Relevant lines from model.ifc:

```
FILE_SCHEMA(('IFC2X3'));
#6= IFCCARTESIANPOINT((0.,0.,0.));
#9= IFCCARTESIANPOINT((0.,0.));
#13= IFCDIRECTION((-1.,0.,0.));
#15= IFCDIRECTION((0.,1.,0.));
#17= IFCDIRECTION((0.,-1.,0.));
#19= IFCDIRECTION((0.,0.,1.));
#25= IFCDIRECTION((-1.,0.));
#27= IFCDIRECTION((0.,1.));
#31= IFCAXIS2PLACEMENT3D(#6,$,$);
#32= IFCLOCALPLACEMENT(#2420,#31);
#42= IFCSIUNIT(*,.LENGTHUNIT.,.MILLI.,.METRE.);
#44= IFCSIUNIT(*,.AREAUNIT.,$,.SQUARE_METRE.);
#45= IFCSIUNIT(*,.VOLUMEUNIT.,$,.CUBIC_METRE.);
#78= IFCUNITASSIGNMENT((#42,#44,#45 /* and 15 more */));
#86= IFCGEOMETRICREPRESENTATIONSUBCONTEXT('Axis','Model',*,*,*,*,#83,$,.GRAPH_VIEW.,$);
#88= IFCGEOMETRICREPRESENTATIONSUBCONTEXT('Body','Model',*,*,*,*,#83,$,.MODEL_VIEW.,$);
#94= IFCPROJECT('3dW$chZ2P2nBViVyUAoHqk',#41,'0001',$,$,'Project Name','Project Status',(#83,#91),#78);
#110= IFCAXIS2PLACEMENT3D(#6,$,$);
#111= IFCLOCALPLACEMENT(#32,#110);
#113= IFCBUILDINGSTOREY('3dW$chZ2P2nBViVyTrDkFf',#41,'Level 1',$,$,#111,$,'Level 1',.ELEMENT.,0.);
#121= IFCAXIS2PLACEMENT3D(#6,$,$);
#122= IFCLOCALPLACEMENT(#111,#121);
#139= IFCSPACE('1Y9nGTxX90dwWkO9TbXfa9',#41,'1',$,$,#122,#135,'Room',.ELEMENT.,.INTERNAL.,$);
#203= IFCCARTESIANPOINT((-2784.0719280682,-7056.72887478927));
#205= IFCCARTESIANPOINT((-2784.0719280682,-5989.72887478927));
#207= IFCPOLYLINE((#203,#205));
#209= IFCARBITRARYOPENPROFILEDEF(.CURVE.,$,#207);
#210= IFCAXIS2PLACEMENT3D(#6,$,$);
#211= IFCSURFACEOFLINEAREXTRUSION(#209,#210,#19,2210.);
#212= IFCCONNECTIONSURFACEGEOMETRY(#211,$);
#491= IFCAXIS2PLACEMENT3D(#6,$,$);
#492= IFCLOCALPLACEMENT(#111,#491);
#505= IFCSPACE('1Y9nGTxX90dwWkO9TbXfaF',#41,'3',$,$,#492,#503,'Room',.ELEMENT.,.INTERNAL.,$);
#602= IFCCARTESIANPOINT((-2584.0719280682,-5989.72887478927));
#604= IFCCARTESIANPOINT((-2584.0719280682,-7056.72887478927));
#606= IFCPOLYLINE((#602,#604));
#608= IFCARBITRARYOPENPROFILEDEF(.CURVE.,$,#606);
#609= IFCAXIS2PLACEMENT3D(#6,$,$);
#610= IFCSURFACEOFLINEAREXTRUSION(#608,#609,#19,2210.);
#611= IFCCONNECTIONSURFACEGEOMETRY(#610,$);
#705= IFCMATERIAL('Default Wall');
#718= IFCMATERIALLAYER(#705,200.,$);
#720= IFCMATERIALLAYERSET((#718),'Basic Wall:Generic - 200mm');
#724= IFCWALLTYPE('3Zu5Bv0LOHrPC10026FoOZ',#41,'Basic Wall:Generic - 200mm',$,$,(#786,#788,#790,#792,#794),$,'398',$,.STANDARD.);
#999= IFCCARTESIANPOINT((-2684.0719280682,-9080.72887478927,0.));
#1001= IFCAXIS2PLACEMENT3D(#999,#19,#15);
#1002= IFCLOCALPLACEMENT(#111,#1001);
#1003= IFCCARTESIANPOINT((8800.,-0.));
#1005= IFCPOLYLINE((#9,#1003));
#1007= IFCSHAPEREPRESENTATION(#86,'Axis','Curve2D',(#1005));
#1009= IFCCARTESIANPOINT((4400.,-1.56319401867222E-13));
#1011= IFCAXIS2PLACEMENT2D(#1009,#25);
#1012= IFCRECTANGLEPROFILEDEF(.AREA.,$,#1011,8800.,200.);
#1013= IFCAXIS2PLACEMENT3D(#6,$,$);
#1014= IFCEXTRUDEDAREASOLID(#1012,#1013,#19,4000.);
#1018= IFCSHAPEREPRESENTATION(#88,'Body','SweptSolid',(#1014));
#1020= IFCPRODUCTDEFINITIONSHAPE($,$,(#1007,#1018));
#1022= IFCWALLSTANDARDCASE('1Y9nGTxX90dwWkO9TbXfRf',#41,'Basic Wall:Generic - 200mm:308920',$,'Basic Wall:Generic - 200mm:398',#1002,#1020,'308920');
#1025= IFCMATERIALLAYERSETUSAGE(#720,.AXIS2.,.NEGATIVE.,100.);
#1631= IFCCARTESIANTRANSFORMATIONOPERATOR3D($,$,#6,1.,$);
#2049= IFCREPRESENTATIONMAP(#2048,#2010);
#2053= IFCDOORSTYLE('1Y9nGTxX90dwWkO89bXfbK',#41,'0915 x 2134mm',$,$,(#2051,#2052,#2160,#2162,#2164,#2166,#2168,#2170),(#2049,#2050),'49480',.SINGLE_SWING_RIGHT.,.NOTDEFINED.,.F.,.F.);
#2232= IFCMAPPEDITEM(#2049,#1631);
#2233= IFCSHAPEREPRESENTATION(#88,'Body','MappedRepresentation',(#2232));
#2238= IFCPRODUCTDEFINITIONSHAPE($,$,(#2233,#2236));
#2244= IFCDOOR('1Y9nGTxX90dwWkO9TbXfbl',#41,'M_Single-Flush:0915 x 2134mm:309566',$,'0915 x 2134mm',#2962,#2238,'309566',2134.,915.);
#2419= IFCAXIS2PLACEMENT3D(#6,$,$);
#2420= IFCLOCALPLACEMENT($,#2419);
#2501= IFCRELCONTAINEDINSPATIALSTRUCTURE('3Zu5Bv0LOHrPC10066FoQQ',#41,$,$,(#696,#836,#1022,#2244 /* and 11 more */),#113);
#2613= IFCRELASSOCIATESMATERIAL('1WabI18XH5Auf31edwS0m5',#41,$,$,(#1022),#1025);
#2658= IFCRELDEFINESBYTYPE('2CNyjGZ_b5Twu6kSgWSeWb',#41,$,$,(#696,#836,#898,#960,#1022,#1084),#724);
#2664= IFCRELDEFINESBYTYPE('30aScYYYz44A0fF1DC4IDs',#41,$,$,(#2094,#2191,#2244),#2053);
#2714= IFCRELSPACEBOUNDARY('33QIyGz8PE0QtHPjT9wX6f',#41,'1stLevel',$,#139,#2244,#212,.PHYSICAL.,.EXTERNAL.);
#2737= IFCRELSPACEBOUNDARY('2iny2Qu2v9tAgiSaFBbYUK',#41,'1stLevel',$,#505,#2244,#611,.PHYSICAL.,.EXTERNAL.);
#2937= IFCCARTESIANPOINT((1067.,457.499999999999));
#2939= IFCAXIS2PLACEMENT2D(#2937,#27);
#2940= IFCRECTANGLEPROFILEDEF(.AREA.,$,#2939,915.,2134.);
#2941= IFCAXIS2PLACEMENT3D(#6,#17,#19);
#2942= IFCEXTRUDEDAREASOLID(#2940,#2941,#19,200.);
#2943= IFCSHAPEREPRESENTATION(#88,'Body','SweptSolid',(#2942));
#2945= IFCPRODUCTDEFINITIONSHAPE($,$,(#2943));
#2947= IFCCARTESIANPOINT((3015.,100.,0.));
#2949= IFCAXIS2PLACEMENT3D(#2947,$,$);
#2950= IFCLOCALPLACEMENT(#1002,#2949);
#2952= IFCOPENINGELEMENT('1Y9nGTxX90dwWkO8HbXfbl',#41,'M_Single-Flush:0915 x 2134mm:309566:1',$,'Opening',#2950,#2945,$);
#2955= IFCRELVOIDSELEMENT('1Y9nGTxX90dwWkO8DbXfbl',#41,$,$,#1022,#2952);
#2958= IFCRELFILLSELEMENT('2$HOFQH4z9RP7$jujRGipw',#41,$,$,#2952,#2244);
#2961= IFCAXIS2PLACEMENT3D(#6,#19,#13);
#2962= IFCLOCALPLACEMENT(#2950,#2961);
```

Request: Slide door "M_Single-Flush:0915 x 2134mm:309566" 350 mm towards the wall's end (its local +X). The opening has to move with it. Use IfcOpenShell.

```python
import numpy as np
import ifcopenshell
import ifcopenshell.api.geometry
import ifcopenshell.util.placement
import ifcopenshell.util.unit

model = ifcopenshell.open("model.ifc")
unit_scale = ifcopenshell.util.unit.calculate_unit_scale(model)

door = model.by_guid("1Y9nGTxX90dwWkO9TbXfbl")
opening = door.FillsVoids[0].RelatingOpeningElement
wall = opening.VoidsElements[0].RelatingBuildingElement

wall_matrix = ifcopenshell.util.placement.get_local_placement(wall.ObjectPlacement)
shift = wall_matrix[:3, 0] * 0.35 / unit_scale
before = ifcopenshell.util.placement.get_local_placement(door.ObjectPlacement)[:3, 3].copy()

# The door is placed relative to its opening, so it follows when the opening moves.
matrix = ifcopenshell.util.placement.get_local_placement(opening.ObjectPlacement)
matrix[:3, 3] += shift
ifcopenshell.api.geometry.edit_object_placement(
    model, product=opening, matrix=matrix, is_si=False, should_transform_children=True
)

# Space boundary surfaces are stored in each space's coordinates; move them too.
for rel in door.ProvidesBoundaries:
    if not rel.ConnectionGeometry:
        continue
    surface = rel.ConnectionGeometry.SurfaceOnRelatingElement
    space_matrix = ifcopenshell.util.placement.get_local_placement(rel.RelatingSpace.ObjectPlacement)
    point = np.array(surface.Position.Location.Coordinates) + space_matrix[:3, :3].T @ shift
    surface.Position = model.createIfcAxis2Placement3D(
        model.createIfcCartesianPoint(point.tolist()), surface.Position.Axis, surface.Position.RefDirection
    )

after = ifcopenshell.util.placement.get_local_placement(door.ObjectPlacement)[:3, 3]
print("door moved by", (after - before).round(3) + 0.0)

model.write("model-out.ifc")
```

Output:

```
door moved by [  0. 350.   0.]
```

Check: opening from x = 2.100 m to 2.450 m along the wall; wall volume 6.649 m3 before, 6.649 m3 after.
